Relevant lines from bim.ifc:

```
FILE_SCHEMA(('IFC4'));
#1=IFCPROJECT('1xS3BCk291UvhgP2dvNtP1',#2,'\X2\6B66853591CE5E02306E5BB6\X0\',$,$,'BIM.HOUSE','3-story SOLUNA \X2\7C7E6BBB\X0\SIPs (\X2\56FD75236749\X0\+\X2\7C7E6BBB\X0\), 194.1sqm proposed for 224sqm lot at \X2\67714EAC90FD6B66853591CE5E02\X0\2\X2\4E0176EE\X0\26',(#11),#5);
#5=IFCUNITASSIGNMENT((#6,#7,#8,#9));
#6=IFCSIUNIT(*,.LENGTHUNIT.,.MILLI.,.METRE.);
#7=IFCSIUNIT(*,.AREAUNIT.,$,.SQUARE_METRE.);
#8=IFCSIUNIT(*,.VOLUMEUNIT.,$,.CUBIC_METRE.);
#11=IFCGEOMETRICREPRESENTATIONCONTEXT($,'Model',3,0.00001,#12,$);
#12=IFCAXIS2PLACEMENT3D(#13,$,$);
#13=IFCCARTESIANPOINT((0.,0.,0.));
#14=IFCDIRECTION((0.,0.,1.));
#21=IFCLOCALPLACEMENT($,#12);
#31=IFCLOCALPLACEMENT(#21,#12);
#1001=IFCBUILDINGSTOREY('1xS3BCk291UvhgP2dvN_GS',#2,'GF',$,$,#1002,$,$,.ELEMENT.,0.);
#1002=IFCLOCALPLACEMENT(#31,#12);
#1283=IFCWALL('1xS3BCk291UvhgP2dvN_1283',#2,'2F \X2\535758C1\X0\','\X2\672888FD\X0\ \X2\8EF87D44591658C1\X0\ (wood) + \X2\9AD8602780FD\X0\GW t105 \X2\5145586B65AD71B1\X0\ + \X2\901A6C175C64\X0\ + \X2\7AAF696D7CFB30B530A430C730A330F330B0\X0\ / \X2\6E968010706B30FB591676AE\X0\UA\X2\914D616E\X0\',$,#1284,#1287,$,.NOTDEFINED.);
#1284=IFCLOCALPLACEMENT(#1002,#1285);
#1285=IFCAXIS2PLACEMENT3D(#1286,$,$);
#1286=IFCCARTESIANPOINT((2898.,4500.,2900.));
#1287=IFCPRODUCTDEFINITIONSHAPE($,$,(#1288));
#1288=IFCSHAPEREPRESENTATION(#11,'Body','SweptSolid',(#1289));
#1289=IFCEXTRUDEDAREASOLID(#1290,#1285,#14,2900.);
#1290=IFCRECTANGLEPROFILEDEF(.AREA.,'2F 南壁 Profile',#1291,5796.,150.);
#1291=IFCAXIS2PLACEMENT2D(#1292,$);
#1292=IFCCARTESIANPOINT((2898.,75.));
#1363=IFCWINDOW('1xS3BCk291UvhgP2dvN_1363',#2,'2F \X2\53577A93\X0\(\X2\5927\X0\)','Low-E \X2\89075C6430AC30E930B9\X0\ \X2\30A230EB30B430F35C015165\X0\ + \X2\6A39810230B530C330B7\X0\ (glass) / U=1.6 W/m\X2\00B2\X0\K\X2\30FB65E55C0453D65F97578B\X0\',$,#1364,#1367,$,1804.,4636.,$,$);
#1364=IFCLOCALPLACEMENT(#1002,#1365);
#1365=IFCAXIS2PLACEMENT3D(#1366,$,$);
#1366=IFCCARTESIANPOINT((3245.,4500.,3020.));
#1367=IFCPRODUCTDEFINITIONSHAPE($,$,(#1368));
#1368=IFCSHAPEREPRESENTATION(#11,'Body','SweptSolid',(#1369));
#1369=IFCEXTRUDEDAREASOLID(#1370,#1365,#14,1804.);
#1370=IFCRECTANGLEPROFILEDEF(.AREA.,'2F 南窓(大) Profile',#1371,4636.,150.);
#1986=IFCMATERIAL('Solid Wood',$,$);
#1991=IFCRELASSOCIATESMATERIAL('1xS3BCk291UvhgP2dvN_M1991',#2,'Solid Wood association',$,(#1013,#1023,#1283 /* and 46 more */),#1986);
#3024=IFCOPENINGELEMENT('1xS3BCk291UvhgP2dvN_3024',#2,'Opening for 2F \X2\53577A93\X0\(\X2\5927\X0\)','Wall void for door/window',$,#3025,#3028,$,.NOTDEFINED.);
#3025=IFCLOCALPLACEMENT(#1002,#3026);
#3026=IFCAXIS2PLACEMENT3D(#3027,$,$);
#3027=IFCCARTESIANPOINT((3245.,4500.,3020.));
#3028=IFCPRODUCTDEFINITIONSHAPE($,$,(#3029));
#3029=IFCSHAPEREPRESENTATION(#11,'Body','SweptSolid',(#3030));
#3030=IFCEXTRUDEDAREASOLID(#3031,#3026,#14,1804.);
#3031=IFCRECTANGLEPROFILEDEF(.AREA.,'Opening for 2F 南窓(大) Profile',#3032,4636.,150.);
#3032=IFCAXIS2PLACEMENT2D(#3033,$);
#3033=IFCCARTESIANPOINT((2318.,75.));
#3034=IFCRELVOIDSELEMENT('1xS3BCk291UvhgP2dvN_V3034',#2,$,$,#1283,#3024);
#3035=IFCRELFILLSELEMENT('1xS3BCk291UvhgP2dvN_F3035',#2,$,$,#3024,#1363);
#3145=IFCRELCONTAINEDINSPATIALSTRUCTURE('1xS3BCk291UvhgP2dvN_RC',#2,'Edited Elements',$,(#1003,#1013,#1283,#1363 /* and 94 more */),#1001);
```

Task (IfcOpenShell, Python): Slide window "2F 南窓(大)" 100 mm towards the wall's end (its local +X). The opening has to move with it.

```python
import ifcopenshell
import ifcopenshell.api.geometry
import ifcopenshell.util.placement

model = ifcopenshell.open("bim.ifc")

window = model.by_id(1363)
opening = window.FillsVoids[0].RelatingOpeningElement
wall = opening.VoidsElements[0].RelatingBuildingElement

wall_matrix = ifcopenshell.util.placement.get_local_placement(wall.ObjectPlacement)
shift = wall_matrix[:3, 0] * 100.0
before = ifcopenshell.util.placement.get_local_placement(window.ObjectPlacement)[:3, 3].copy()

# The window is not placed relative to its opening, so move both.
for product in (opening, window):
    matrix = ifcopenshell.util.placement.get_local_placement(product.ObjectPlacement)
    matrix[:3, 3] += shift
    ifcopenshell.api.geometry.edit_object_placement(model, product=product, matrix=matrix, is_si=False)

after = ifcopenshell.util.placement.get_local_placement(window.ObjectPlacement)[:3, 3]
print("window moved by", (after - before).round(3) + 0.0)

model.write("bim-out.ifc")
```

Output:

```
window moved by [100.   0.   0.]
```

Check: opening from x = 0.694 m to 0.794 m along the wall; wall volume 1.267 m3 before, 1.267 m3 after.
